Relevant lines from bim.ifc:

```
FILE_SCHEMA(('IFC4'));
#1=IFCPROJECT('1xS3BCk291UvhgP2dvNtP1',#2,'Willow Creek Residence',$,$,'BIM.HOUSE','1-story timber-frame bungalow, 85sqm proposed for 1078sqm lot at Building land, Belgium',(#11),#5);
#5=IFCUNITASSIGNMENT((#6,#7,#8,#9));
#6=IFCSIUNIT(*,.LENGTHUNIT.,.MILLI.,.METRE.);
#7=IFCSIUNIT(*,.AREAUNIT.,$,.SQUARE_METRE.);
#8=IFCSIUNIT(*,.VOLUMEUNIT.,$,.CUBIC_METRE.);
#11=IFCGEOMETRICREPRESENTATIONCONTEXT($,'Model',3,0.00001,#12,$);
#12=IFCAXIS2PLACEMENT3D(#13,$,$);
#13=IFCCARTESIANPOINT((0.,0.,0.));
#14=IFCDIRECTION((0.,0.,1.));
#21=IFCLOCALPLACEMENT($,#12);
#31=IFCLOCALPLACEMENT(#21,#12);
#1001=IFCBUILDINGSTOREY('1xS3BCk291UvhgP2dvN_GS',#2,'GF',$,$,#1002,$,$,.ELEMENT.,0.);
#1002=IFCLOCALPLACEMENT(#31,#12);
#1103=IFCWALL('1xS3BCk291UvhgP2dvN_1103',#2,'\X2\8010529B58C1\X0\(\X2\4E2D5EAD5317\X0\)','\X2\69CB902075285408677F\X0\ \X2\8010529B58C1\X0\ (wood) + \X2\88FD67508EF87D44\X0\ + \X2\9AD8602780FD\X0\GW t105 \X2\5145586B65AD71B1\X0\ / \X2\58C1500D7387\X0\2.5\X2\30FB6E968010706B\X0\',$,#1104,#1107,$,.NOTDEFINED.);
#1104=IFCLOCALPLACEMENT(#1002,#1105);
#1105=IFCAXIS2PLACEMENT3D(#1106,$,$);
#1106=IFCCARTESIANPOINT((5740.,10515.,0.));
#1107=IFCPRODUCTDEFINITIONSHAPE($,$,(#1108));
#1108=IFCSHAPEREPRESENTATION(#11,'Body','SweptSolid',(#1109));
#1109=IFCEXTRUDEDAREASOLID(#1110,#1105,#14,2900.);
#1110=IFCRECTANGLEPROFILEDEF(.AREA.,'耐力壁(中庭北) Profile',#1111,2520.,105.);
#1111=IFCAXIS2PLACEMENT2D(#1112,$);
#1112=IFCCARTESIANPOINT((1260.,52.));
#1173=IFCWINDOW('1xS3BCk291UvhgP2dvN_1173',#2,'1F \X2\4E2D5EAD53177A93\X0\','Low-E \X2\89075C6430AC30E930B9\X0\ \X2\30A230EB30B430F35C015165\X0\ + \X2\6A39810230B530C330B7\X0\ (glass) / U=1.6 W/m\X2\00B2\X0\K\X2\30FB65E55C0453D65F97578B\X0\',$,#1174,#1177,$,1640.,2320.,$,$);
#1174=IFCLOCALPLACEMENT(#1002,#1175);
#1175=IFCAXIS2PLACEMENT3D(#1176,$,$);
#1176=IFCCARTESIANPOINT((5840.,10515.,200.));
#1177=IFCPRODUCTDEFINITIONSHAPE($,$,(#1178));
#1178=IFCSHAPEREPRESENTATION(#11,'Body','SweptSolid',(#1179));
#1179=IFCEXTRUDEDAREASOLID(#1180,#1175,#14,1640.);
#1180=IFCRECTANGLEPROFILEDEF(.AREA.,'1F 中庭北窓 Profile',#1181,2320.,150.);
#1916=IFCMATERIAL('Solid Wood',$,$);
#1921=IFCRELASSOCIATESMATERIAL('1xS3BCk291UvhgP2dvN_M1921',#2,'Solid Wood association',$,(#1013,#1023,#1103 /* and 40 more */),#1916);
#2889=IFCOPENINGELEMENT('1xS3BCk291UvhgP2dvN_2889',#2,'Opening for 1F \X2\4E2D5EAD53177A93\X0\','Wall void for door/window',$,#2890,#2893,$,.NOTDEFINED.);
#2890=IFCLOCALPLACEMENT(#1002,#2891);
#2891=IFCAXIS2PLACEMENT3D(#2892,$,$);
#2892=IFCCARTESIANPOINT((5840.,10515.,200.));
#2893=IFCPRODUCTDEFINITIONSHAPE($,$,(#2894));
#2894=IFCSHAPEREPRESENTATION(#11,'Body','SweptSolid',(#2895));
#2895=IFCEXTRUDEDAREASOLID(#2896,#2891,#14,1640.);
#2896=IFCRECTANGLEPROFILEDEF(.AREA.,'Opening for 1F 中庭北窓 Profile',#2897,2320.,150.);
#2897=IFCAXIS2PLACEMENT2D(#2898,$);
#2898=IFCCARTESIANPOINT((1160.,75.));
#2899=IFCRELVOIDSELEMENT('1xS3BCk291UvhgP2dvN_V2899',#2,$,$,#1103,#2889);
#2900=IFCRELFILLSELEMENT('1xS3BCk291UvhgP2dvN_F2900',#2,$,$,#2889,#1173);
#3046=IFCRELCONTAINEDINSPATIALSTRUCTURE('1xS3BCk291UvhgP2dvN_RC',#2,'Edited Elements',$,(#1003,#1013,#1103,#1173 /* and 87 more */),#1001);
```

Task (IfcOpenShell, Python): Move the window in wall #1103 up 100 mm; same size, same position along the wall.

```python
import numpy as np
import ifcopenshell
import ifcopenshell.api.geometry
import ifcopenshell.util.placement
import ifcopenshell.util.unit

model = ifcopenshell.open("bim.ifc")
unit_scale = ifcopenshell.util.unit.calculate_unit_scale(model)

window = model.by_guid("1xS3BCk291UvhgP2dvN_1173")
opening = window.FillsVoids[0].RelatingOpeningElement
dz = 0.1 / unit_scale

shift = np.array([0.0, 0.0, dz])
# The window is not placed relative to its opening, so move both.
for product in (opening, window):
    matrix = ifcopenshell.util.placement.get_local_placement(product.ObjectPlacement)
    matrix[:3, 3] += shift
    ifcopenshell.api.geometry.edit_object_placement(model, product=product, matrix=matrix, is_si=False)

print(f"moved by {dz * unit_scale:+.3f} m")

model.write("bim_updated.ifc")
```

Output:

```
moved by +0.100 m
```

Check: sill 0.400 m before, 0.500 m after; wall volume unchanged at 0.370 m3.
